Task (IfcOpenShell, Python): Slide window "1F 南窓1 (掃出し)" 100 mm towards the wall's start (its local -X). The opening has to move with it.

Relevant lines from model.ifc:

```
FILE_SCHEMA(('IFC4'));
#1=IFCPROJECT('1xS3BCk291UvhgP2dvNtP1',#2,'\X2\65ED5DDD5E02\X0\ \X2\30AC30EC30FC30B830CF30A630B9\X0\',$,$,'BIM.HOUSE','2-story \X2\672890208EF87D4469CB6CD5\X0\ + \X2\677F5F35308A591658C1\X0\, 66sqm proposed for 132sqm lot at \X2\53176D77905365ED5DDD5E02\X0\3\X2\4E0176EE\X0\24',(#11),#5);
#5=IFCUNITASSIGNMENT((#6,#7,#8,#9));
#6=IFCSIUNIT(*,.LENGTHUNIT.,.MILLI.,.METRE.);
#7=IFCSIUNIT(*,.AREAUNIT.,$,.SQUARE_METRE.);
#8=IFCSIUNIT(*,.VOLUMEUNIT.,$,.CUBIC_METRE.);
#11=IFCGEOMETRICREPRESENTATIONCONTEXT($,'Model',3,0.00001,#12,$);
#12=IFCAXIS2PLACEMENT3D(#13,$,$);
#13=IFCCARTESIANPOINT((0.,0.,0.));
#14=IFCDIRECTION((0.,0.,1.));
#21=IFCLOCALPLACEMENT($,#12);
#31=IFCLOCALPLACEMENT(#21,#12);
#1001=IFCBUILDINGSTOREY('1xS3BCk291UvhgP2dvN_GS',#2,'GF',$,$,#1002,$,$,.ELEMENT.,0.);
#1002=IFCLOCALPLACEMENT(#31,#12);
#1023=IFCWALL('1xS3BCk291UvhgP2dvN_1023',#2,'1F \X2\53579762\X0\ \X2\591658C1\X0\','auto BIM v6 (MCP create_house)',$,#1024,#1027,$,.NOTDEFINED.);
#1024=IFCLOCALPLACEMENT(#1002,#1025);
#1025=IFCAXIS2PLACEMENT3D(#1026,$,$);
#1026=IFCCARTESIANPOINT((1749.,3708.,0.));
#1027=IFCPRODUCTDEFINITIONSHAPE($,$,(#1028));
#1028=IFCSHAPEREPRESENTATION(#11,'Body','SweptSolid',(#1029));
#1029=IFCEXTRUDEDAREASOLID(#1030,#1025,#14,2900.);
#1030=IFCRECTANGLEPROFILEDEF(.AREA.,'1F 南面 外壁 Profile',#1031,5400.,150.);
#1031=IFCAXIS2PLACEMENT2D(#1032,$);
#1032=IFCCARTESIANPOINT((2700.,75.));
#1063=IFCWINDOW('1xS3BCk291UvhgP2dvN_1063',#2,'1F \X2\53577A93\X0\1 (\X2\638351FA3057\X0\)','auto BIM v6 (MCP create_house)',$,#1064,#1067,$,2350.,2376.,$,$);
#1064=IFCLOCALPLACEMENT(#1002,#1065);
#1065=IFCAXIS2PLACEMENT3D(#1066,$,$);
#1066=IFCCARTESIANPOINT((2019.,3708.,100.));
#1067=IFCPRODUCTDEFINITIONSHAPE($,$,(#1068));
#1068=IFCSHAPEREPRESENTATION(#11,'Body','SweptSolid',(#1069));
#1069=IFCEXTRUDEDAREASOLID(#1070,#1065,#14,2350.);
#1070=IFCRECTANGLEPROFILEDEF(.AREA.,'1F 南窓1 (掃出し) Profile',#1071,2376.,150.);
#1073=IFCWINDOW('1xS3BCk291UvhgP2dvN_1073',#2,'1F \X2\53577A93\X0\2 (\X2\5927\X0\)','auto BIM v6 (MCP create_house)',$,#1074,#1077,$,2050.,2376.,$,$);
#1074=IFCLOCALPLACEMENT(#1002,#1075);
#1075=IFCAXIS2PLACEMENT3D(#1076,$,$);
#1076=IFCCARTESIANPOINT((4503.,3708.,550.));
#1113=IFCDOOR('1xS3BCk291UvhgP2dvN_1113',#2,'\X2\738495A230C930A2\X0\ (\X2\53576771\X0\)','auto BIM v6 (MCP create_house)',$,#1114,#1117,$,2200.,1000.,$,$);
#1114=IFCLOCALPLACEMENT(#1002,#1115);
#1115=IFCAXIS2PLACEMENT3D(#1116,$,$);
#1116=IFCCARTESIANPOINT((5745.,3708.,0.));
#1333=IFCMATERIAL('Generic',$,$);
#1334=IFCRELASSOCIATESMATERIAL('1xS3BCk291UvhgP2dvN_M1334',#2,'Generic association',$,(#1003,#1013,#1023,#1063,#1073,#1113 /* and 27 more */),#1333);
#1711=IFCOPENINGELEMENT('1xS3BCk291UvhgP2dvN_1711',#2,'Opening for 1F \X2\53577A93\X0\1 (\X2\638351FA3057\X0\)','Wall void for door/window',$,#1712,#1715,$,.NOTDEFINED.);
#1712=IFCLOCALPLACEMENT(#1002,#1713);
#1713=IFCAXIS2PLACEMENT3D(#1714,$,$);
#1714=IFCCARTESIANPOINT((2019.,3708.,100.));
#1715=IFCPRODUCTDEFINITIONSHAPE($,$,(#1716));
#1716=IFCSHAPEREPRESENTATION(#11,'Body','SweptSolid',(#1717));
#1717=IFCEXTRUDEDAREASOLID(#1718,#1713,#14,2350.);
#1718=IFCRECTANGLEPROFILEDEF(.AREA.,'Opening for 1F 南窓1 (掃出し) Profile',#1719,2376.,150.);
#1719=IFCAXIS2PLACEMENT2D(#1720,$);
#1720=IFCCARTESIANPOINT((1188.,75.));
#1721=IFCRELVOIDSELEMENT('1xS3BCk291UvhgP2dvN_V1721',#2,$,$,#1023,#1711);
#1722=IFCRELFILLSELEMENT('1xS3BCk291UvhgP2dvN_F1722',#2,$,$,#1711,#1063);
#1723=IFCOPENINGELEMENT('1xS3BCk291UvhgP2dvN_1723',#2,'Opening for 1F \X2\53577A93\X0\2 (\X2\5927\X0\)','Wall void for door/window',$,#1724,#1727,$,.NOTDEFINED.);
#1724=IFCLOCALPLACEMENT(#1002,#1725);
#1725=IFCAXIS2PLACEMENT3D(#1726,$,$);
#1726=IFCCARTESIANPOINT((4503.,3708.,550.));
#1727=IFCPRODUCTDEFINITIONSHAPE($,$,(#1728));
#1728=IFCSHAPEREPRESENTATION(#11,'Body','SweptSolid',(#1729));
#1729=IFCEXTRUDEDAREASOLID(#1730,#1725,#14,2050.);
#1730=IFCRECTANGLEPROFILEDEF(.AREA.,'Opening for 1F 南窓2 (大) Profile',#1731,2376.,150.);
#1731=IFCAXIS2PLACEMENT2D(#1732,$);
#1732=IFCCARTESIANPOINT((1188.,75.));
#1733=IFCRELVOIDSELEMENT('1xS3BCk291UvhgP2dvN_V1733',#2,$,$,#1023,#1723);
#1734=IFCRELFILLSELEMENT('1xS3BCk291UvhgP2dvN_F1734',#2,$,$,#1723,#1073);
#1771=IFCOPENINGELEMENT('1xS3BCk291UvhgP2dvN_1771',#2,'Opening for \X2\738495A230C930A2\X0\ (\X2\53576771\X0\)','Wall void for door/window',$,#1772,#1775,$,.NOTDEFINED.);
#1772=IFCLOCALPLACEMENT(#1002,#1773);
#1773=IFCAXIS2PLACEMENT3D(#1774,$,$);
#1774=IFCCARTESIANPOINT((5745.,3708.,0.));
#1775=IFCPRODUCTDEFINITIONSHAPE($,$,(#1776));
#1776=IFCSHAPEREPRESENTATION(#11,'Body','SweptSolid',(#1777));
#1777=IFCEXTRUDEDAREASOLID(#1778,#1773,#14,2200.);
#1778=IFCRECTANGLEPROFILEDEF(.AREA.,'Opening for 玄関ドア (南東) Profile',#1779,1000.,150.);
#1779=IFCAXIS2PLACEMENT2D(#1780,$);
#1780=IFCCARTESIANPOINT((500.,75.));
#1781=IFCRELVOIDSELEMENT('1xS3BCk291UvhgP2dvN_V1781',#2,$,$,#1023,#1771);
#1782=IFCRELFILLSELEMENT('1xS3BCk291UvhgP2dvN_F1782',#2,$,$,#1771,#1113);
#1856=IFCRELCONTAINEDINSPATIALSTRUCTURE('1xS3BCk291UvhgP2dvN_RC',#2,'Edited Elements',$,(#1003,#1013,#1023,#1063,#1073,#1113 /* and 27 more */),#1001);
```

```python
import ifcopenshell
import ifcopenshell.api.geometry
import ifcopenshell.util.placement

model = ifcopenshell.open("model.ifc")

window = model.by_id(1063)
opening = window.FillsVoids[0].RelatingOpeningElement
wall = opening.VoidsElements[0].RelatingBuildingElement

wall_matrix = ifcopenshell.util.placement.get_local_placement(wall.ObjectPlacement)
shift = wall_matrix[:3, 0] * -100.0
before = ifcopenshell.util.placement.get_local_placement(window.ObjectPlacement)[:3, 3].copy()

# The window is not placed relative to its opening, so move both.
for product in (opening, window):
    matrix = ifcopenshell.util.placement.get_local_placement(product.ObjectPlacement)
    matrix[:3, 3] += shift
    ifcopenshell.api.geometry.edit_object_placement(model, product=product, matrix=matrix, is_si=False)

after = ifcopenshell.util.placement.get_local_placement(window.ObjectPlacement)[:3, 3]
print("window moved by", (after - before).round(3) + 0.0)

model.write("model_v2.ifc")
```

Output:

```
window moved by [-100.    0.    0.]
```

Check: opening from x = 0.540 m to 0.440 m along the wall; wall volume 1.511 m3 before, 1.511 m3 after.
